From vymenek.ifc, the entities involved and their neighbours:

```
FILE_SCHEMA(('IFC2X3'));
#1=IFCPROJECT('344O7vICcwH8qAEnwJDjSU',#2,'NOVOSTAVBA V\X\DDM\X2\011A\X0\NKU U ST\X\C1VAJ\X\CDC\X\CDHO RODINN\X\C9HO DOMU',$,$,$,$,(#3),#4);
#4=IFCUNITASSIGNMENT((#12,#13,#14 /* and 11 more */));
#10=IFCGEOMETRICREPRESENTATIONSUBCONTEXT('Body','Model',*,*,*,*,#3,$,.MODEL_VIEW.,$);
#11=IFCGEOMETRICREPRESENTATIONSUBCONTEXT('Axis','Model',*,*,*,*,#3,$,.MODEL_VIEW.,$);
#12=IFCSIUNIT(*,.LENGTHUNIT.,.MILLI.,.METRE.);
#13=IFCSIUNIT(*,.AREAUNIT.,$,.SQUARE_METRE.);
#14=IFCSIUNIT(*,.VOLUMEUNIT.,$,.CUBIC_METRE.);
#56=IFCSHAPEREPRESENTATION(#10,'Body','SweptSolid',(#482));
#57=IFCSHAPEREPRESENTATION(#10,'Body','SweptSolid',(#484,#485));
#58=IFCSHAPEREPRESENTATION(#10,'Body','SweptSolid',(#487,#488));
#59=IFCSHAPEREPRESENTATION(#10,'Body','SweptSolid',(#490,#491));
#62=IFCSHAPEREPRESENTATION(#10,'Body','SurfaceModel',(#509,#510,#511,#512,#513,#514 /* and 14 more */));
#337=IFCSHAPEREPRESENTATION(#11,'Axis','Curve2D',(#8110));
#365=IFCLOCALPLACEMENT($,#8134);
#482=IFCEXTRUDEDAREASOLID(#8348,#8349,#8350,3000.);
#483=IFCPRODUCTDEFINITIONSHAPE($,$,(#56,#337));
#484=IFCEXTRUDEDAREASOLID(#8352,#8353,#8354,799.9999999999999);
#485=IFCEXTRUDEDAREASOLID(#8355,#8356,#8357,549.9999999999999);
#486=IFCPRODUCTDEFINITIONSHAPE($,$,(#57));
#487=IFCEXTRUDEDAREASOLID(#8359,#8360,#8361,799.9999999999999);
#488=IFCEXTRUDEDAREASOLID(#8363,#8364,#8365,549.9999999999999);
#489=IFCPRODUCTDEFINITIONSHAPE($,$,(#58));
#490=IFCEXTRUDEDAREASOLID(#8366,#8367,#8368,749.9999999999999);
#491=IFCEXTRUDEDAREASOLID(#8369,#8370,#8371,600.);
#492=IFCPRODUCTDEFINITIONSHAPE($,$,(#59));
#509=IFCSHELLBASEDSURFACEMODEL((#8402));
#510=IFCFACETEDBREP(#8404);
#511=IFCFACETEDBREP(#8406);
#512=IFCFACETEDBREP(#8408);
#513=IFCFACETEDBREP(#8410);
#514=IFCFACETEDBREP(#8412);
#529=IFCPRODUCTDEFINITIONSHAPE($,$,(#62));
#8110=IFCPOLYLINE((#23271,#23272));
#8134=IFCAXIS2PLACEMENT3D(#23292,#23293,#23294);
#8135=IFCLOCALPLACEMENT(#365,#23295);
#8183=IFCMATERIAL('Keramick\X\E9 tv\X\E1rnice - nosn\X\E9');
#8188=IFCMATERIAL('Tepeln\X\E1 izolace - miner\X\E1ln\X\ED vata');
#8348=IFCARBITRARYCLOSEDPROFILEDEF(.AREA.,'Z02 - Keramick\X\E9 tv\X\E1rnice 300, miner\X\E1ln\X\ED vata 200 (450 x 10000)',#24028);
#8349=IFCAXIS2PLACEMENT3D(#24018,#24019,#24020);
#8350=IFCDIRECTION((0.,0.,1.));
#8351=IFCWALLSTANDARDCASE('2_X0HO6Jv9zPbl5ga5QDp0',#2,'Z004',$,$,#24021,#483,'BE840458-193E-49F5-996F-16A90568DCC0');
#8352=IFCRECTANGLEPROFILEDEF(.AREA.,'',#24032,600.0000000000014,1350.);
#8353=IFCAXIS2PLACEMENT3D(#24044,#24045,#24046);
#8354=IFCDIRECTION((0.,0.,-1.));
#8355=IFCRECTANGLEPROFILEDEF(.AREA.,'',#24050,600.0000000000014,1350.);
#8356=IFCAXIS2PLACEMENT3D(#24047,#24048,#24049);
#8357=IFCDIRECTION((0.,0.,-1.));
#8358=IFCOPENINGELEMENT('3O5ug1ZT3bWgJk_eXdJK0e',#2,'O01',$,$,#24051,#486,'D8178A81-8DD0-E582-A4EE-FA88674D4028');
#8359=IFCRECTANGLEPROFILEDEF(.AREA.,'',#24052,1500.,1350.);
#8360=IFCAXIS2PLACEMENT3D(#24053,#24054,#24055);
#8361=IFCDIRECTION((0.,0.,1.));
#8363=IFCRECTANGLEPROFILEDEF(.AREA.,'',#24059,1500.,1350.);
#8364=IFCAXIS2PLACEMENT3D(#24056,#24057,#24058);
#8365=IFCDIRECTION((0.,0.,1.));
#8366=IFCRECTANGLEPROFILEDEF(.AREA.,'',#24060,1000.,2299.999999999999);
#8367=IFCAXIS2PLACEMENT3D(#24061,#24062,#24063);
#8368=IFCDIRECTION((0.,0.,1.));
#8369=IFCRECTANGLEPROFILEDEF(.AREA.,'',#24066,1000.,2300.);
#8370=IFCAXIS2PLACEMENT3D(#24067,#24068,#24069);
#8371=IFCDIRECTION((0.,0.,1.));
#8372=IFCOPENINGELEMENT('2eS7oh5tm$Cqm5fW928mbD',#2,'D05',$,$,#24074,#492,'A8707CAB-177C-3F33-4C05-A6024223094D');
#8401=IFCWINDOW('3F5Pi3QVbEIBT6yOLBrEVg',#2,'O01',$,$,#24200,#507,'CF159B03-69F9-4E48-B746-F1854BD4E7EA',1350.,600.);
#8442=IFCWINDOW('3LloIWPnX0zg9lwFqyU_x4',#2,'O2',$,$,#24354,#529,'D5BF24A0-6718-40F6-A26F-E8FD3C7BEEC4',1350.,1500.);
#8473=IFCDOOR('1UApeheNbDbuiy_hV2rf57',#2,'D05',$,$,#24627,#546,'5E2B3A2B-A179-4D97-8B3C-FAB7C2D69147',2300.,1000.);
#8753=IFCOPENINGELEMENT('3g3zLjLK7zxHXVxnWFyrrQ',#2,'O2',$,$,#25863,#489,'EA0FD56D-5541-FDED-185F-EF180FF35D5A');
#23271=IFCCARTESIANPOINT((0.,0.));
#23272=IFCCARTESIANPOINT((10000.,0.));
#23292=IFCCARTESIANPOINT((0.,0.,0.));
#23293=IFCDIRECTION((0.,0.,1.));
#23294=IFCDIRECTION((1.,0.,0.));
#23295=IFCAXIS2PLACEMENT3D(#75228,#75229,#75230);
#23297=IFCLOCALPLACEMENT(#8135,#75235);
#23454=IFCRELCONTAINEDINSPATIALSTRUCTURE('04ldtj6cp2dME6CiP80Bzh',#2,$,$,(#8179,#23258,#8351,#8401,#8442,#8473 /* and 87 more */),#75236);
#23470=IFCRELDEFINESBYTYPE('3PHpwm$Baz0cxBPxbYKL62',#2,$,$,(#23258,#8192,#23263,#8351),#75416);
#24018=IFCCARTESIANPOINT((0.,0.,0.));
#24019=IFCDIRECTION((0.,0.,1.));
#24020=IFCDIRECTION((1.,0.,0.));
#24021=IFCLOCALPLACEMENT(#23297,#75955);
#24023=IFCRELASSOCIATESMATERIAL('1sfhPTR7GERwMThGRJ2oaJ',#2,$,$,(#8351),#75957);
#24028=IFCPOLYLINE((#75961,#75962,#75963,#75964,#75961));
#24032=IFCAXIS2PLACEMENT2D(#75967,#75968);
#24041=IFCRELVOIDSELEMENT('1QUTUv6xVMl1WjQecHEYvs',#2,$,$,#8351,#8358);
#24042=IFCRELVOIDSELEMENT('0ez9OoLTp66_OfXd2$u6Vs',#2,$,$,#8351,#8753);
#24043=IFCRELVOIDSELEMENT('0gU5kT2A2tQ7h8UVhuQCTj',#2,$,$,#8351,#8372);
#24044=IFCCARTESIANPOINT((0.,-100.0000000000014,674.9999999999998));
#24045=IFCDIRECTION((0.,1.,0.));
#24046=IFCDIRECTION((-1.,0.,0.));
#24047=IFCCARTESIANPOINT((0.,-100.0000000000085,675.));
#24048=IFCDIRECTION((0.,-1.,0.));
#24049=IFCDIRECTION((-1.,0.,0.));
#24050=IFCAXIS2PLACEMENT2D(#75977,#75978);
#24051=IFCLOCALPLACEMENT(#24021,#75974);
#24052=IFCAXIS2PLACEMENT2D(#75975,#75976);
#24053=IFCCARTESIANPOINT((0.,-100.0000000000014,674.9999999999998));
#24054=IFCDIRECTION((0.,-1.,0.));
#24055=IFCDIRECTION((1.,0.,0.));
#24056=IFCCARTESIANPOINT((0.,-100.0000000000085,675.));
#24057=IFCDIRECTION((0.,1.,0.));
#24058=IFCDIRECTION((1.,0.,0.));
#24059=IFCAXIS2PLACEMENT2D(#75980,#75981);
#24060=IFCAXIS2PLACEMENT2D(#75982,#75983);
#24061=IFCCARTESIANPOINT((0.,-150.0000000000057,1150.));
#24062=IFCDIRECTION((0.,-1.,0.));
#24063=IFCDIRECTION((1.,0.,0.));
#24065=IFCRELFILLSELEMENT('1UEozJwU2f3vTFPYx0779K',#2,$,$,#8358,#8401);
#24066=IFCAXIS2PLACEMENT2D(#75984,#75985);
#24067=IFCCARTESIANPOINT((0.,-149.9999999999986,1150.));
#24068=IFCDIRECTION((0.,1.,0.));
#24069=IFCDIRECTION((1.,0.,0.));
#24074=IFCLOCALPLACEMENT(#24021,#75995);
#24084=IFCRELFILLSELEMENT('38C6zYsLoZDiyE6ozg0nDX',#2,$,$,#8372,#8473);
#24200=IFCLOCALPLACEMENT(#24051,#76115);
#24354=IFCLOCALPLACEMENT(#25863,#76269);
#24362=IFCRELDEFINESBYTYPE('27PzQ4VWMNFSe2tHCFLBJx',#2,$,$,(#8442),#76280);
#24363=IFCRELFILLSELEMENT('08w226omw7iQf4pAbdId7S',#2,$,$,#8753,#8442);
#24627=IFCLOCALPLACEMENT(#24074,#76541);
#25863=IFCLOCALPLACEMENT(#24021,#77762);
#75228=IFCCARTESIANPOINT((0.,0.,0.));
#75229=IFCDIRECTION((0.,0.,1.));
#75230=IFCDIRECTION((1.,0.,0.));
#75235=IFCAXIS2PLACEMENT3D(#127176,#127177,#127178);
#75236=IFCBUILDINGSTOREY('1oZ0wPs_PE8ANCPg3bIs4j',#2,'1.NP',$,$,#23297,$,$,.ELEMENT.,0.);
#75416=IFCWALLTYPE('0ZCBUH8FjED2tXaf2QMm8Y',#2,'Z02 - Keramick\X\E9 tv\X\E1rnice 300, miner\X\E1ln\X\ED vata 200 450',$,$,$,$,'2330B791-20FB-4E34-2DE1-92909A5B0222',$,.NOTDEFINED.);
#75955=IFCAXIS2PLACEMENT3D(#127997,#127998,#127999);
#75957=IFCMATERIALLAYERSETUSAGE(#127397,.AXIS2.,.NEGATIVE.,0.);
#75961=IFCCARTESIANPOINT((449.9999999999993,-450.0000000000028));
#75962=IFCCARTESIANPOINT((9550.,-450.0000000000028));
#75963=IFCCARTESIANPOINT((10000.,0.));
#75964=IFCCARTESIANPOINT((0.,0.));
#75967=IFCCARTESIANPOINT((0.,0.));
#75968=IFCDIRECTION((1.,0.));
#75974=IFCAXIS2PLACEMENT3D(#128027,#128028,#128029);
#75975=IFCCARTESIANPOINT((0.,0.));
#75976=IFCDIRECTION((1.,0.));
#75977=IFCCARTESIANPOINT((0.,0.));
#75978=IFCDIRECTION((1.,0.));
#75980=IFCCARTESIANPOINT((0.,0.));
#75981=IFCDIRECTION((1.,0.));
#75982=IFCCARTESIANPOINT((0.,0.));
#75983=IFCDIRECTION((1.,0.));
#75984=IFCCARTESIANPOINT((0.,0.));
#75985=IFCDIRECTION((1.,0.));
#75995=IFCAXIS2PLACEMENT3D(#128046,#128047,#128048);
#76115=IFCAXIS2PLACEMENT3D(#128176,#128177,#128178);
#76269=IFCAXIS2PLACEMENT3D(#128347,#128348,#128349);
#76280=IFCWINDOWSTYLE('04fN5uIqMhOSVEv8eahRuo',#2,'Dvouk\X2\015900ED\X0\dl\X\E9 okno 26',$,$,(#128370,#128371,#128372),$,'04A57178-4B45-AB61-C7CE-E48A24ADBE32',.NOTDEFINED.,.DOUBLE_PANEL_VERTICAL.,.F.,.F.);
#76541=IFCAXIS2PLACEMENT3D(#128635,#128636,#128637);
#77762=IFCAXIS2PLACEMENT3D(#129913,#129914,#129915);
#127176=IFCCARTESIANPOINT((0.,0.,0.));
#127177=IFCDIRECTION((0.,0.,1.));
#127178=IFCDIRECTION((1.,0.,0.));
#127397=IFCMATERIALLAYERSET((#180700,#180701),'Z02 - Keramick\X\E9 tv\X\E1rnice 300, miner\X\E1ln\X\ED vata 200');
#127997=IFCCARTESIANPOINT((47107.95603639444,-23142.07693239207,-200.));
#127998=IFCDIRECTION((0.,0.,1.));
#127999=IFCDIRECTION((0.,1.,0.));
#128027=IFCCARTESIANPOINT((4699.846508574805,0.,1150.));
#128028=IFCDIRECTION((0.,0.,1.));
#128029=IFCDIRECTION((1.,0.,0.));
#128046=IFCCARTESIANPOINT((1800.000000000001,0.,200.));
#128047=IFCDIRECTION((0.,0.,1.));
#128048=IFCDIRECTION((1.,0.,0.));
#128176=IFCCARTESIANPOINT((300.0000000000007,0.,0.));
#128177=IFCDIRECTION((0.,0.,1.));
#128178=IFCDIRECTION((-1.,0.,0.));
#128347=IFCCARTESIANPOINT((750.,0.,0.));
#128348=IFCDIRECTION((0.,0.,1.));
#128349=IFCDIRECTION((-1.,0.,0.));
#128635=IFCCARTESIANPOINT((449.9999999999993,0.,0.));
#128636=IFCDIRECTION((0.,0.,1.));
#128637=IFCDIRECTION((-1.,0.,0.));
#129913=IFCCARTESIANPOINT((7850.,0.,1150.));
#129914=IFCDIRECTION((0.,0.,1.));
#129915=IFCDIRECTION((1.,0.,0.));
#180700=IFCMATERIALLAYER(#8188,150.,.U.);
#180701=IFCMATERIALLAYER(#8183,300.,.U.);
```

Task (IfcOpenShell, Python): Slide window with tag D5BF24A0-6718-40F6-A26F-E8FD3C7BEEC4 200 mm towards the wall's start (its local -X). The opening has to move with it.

```python
import ifcopenshell
import ifcopenshell.api.geometry
import ifcopenshell.util.placement
import ifcopenshell.util.unit

model = ifcopenshell.open("vymenek.ifc")
unit_scale = ifcopenshell.util.unit.calculate_unit_scale(model)

window = model.by_guid("3LloIWPnX0zg9lwFqyU_x4")
opening = window.FillsVoids[0].RelatingOpeningElement
wall = opening.VoidsElements[0].RelatingBuildingElement

wall_matrix = ifcopenshell.util.placement.get_local_placement(wall.ObjectPlacement)
shift = wall_matrix[:3, 0] * -0.2 / unit_scale
before = ifcopenshell.util.placement.get_local_placement(window.ObjectPlacement)[:3, 3].copy()

# The window is placed relative to its opening, so it follows when the opening moves.
matrix = ifcopenshell.util.placement.get_local_placement(opening.ObjectPlacement)
matrix[:3, 3] += shift
ifcopenshell.api.geometry.edit_object_placement(
    model, product=opening, matrix=matrix, is_si=False, should_transform_children=True
)

after = ifcopenshell.util.placement.get_local_placement(window.ObjectPlacement)[:3, 3]
print("window moved by", (after - before).round(3) + 0.0)

model.write("vymenek_rev.ifc")
```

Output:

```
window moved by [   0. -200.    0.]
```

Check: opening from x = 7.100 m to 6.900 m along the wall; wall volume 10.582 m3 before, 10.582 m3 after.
